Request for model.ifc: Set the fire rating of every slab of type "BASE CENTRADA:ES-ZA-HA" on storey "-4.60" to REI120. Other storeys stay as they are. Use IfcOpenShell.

First a look at what the model holds.

```python
import ifcopenshell
import ifcopenshell.util.element

model = ifcopenshell.open("model.ifc")
print(model.schema)
storey = next(s for s in model.by_type("IfcBuildingStorey") if s.Name == "-4.60")
slabs = [e for e in ifcopenshell.util.element.get_decomposition(storey) if e.is_a("IfcSlab")]
seen = {}
for e in slabs:
    element_type = ifcopenshell.util.element.get_type(e)
    key = (element_type.Name if element_type != e and element_type else None, ifcopenshell.util.element.get_pset(e, "Pset_SlabCommon", "FireRating"))
    seen[key] = seen.get(key, 0) + 1
for (name, value), count in sorted(seen.items(), key=str):
    print(count, "x", name, "|", value)
```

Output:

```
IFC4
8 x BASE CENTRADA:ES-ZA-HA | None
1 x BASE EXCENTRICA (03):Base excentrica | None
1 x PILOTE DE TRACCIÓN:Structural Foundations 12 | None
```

```python
import ifcopenshell
import ifcopenshell.api.pset
import ifcopenshell.util.element

model = ifcopenshell.open("model.ifc")

storey = next(s for s in model.by_type("IfcBuildingStorey") if s.Name == "-4.60")
slabs = [e for e in ifcopenshell.util.element.get_decomposition(storey) if e.is_a("IfcSlab")]

count = 0
for e in slabs:
    element_type = ifcopenshell.util.element.get_type(e)
    if element_type in (None, e) or element_type.Name != "BASE CENTRADA:ES-ZA-HA":
        continue
    # add_pset returns the element's existing set when there is one.
    pset = ifcopenshell.api.pset.add_pset(model, product=e, name="Pset_SlabCommon")
    ifcopenshell.api.pset.edit_pset(model, pset=pset, properties={"FireRating": "REI120"})
    count += 1

print(count, "slabs updated")

model.write("model_updated.ifc")
```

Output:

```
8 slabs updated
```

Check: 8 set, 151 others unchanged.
